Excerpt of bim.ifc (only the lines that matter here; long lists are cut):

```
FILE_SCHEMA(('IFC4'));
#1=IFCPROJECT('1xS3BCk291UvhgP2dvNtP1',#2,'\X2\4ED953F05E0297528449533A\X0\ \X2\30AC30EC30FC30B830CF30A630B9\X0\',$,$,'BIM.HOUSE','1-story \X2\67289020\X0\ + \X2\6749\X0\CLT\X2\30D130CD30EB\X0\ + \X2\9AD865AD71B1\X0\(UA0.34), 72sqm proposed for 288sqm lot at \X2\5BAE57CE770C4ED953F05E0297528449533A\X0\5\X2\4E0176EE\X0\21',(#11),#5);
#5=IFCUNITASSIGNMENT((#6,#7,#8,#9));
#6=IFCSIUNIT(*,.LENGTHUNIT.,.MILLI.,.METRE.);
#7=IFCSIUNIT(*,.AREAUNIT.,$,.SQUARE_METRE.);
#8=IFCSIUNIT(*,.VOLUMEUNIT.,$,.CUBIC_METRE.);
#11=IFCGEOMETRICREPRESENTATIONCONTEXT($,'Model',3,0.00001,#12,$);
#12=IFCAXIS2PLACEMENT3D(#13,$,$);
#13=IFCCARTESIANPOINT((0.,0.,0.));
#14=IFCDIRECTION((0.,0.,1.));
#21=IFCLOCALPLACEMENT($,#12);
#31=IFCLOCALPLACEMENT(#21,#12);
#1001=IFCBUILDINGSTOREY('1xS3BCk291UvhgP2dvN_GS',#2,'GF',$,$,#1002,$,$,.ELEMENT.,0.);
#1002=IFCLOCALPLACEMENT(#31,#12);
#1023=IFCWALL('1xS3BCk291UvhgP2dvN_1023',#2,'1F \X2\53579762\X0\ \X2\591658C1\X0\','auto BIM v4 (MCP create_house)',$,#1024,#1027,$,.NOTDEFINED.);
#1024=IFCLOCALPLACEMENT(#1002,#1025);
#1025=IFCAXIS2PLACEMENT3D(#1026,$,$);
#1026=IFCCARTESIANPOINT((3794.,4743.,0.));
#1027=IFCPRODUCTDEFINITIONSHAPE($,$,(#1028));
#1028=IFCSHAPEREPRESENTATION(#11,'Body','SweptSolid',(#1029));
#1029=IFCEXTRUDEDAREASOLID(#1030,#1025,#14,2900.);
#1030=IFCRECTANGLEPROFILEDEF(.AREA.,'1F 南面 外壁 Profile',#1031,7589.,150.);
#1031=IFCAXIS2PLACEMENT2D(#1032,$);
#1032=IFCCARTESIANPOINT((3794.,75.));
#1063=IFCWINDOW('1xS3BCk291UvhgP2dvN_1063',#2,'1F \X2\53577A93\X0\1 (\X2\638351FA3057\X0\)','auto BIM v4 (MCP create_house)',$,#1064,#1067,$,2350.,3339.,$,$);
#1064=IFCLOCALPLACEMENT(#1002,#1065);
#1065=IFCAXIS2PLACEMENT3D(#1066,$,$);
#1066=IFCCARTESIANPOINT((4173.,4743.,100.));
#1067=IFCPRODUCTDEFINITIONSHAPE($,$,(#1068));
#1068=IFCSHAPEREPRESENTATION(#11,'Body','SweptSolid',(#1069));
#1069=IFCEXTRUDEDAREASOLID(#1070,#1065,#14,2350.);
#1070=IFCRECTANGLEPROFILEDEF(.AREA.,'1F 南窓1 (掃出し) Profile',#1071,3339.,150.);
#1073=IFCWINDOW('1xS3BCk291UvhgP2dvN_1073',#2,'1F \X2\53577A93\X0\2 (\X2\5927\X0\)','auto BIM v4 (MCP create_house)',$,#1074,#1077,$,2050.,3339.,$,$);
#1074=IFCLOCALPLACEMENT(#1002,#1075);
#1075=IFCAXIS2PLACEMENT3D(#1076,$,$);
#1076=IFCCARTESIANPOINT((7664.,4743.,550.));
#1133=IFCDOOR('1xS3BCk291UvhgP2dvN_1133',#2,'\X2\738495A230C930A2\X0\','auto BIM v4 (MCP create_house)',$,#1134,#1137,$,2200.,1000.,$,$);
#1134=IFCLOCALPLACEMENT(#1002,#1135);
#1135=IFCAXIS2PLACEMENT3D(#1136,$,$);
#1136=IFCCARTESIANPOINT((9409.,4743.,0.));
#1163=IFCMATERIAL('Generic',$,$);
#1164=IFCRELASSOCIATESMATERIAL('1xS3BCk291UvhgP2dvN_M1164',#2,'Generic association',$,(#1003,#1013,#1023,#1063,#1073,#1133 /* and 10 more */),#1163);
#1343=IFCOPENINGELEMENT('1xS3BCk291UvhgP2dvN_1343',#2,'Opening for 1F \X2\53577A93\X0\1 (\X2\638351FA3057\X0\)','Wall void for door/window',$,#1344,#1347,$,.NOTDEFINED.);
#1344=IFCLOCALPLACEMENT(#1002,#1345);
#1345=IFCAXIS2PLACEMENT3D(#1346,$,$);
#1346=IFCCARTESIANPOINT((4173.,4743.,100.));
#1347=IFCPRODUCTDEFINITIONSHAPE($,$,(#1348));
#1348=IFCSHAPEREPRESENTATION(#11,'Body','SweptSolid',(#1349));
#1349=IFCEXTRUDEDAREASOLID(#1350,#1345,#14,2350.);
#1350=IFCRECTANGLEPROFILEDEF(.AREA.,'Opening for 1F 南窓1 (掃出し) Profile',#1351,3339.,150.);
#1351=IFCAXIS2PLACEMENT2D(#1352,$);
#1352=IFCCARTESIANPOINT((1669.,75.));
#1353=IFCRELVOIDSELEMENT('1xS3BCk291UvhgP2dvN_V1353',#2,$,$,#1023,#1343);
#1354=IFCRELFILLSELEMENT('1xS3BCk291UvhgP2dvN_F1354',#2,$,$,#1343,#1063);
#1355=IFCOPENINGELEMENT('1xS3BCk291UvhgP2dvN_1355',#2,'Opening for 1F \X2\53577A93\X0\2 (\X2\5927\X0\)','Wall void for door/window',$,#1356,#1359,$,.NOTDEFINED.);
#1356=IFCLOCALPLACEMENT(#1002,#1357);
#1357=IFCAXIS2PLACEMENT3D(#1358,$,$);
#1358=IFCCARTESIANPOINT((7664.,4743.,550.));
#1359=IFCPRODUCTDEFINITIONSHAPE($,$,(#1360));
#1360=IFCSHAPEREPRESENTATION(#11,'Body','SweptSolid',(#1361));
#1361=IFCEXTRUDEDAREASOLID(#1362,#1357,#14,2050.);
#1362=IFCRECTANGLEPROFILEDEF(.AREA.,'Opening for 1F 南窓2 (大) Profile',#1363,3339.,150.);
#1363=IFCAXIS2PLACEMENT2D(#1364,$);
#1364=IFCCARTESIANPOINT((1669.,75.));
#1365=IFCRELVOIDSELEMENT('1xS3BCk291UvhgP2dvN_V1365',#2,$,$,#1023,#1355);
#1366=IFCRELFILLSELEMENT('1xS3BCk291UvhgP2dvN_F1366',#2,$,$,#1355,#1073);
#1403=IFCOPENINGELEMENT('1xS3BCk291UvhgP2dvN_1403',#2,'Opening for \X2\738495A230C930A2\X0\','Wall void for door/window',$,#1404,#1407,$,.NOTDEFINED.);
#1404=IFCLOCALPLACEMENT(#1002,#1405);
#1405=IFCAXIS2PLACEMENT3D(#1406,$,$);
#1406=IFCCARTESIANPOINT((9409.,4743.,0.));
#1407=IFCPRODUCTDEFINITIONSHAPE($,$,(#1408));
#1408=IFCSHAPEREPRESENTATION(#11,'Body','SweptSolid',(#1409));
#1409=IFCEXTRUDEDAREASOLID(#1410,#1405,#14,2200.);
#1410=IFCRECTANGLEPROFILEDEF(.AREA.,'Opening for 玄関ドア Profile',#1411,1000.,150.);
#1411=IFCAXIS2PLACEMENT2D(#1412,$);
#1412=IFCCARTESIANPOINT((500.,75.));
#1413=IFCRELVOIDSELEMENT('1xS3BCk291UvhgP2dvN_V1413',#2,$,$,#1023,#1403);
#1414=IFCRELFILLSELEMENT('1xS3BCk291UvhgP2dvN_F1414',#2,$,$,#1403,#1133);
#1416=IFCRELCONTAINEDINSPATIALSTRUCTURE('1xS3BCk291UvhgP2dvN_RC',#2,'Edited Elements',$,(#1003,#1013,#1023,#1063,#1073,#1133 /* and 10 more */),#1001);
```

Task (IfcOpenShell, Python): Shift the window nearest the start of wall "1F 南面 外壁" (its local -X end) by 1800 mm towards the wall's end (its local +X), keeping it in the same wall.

```python
import ifcopenshell
import ifcopenshell.api.geometry
import ifcopenshell.util.placement
import ifcopenshell.util.unit

model = ifcopenshell.open("bim.ifc")
unit_scale = ifcopenshell.util.unit.calculate_unit_scale(model)

window = model.by_guid("1xS3BCk291UvhgP2dvN_1063")
opening = window.FillsVoids[0].RelatingOpeningElement
wall = opening.VoidsElements[0].RelatingBuildingElement

wall_matrix = ifcopenshell.util.placement.get_local_placement(wall.ObjectPlacement)
shift = wall_matrix[:3, 0] * 1.8 / unit_scale
before = ifcopenshell.util.placement.get_local_placement(window.ObjectPlacement)[:3, 3].copy()

# The window is not placed relative to its opening, so move both.
for product in (opening, window):
    matrix = ifcopenshell.util.placement.get_local_placement(product.ObjectPlacement)
    matrix[:3, 3] += shift
    ifcopenshell.api.geometry.edit_object_placement(model, product=product, matrix=matrix, is_si=False)

after = ifcopenshell.util.placement.get_local_placement(window.ObjectPlacement)[:3, 3]
print("window moved by", (after - before).round(3) + 0.0)

model.write("bim_edited.ifc")
```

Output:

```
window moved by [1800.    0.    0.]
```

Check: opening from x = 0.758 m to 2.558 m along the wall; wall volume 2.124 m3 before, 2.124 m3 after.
